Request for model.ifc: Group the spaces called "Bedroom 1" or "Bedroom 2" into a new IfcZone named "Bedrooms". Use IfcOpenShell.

First a look at what the model holds.

```python
import ifcopenshell

model = ifcopenshell.open("model.ifc")
print(model.schema)
seen = {}
for space in model.by_type("IfcSpace"):
    seen[space.LongName] = seen.get(space.LongName, 0) + 1
for name, count in sorted(seen.items(), key=str):
    print(count, "x", name)
print("zones:", [z.Name for z in model.by_type("IfcZone")][:20])
```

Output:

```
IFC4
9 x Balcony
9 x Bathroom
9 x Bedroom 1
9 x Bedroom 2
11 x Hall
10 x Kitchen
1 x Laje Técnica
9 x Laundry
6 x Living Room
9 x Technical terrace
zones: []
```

```python
import ifcopenshell
import ifcopenshell.api.group
import ifcopenshell.api.root

model = ifcopenshell.open("model.ifc")

names = {"Bedroom 1", "Bedroom 2"}
spaces = [s for s in model.by_type("IfcSpace") if s.LongName in names]

zone = ifcopenshell.api.root.create_entity(model, ifc_class="IfcZone", name="Bedrooms")
ifcopenshell.api.group.assign_group(model, products=spaces, group=zone)
print(len(spaces), "spaces in", zone.Name)

model.write("model_updated.ifc")
```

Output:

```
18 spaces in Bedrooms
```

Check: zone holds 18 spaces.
